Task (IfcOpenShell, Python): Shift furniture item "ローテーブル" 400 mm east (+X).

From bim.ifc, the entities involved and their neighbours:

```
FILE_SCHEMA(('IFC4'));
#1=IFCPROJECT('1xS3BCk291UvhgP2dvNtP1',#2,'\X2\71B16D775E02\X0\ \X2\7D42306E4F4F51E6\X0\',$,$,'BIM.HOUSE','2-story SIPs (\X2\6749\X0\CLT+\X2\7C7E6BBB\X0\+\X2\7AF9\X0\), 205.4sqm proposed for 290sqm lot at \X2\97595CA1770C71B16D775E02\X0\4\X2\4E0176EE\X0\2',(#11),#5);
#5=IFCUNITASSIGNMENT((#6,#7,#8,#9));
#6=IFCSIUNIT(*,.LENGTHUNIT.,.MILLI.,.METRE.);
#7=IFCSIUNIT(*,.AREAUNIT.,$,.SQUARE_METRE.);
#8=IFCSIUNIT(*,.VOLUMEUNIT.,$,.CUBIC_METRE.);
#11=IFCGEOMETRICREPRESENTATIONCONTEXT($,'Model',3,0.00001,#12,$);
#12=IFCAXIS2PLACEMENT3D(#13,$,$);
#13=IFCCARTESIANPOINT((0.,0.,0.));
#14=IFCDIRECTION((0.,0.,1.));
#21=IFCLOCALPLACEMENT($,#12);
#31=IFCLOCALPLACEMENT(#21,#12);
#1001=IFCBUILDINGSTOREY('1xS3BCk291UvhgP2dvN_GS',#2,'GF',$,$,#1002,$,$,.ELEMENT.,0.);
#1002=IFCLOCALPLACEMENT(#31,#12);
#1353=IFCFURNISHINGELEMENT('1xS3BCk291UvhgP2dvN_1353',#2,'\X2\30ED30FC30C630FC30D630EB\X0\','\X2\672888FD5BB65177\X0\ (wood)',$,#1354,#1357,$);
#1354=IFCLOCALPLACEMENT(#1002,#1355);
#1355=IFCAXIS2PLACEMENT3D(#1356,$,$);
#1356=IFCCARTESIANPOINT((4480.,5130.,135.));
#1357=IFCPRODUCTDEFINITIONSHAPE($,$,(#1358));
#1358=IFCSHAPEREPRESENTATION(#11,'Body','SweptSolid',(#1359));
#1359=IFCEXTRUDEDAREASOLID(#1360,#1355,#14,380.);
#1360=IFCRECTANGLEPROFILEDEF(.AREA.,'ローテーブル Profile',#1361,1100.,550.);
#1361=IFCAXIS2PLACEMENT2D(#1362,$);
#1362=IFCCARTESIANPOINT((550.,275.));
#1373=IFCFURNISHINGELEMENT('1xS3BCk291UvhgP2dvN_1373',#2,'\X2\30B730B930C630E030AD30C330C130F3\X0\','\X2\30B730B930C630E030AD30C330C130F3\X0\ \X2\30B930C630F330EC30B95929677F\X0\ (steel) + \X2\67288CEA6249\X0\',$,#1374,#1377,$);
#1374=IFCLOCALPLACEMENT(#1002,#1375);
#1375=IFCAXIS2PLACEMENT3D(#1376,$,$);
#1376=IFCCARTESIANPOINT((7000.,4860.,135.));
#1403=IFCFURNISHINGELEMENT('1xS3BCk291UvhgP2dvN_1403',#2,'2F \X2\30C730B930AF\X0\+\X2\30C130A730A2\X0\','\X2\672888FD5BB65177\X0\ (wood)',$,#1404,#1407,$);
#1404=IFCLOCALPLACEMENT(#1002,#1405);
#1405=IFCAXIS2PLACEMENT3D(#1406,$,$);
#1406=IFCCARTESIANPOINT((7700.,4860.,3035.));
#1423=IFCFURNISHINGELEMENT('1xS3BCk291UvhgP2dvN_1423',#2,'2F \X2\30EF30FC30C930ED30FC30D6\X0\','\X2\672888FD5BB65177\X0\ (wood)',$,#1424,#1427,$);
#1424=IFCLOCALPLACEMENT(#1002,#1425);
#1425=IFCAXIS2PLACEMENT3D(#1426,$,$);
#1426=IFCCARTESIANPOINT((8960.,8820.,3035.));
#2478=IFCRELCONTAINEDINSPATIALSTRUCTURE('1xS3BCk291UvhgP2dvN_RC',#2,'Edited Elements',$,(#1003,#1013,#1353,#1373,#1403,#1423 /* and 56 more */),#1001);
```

```python
import ifcopenshell
import ifcopenshell.api.geometry
import ifcopenshell.util.placement

model = ifcopenshell.open("bim.ifc")

item = model.by_id(1353)
matrix = ifcopenshell.util.placement.get_local_placement(item.ObjectPlacement)
matrix[0, 3] += 400.0
ifcopenshell.api.geometry.edit_object_placement(model, product=item, matrix=matrix, is_si=False)

print(ifcopenshell.util.placement.get_local_placement(item.ObjectPlacement).round(3) + 0.0)

model.write("bim_updated.ifc")
```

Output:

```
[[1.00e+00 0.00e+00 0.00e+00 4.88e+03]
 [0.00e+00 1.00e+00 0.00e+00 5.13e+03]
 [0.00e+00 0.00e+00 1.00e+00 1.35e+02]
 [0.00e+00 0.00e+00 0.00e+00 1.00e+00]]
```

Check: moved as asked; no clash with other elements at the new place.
